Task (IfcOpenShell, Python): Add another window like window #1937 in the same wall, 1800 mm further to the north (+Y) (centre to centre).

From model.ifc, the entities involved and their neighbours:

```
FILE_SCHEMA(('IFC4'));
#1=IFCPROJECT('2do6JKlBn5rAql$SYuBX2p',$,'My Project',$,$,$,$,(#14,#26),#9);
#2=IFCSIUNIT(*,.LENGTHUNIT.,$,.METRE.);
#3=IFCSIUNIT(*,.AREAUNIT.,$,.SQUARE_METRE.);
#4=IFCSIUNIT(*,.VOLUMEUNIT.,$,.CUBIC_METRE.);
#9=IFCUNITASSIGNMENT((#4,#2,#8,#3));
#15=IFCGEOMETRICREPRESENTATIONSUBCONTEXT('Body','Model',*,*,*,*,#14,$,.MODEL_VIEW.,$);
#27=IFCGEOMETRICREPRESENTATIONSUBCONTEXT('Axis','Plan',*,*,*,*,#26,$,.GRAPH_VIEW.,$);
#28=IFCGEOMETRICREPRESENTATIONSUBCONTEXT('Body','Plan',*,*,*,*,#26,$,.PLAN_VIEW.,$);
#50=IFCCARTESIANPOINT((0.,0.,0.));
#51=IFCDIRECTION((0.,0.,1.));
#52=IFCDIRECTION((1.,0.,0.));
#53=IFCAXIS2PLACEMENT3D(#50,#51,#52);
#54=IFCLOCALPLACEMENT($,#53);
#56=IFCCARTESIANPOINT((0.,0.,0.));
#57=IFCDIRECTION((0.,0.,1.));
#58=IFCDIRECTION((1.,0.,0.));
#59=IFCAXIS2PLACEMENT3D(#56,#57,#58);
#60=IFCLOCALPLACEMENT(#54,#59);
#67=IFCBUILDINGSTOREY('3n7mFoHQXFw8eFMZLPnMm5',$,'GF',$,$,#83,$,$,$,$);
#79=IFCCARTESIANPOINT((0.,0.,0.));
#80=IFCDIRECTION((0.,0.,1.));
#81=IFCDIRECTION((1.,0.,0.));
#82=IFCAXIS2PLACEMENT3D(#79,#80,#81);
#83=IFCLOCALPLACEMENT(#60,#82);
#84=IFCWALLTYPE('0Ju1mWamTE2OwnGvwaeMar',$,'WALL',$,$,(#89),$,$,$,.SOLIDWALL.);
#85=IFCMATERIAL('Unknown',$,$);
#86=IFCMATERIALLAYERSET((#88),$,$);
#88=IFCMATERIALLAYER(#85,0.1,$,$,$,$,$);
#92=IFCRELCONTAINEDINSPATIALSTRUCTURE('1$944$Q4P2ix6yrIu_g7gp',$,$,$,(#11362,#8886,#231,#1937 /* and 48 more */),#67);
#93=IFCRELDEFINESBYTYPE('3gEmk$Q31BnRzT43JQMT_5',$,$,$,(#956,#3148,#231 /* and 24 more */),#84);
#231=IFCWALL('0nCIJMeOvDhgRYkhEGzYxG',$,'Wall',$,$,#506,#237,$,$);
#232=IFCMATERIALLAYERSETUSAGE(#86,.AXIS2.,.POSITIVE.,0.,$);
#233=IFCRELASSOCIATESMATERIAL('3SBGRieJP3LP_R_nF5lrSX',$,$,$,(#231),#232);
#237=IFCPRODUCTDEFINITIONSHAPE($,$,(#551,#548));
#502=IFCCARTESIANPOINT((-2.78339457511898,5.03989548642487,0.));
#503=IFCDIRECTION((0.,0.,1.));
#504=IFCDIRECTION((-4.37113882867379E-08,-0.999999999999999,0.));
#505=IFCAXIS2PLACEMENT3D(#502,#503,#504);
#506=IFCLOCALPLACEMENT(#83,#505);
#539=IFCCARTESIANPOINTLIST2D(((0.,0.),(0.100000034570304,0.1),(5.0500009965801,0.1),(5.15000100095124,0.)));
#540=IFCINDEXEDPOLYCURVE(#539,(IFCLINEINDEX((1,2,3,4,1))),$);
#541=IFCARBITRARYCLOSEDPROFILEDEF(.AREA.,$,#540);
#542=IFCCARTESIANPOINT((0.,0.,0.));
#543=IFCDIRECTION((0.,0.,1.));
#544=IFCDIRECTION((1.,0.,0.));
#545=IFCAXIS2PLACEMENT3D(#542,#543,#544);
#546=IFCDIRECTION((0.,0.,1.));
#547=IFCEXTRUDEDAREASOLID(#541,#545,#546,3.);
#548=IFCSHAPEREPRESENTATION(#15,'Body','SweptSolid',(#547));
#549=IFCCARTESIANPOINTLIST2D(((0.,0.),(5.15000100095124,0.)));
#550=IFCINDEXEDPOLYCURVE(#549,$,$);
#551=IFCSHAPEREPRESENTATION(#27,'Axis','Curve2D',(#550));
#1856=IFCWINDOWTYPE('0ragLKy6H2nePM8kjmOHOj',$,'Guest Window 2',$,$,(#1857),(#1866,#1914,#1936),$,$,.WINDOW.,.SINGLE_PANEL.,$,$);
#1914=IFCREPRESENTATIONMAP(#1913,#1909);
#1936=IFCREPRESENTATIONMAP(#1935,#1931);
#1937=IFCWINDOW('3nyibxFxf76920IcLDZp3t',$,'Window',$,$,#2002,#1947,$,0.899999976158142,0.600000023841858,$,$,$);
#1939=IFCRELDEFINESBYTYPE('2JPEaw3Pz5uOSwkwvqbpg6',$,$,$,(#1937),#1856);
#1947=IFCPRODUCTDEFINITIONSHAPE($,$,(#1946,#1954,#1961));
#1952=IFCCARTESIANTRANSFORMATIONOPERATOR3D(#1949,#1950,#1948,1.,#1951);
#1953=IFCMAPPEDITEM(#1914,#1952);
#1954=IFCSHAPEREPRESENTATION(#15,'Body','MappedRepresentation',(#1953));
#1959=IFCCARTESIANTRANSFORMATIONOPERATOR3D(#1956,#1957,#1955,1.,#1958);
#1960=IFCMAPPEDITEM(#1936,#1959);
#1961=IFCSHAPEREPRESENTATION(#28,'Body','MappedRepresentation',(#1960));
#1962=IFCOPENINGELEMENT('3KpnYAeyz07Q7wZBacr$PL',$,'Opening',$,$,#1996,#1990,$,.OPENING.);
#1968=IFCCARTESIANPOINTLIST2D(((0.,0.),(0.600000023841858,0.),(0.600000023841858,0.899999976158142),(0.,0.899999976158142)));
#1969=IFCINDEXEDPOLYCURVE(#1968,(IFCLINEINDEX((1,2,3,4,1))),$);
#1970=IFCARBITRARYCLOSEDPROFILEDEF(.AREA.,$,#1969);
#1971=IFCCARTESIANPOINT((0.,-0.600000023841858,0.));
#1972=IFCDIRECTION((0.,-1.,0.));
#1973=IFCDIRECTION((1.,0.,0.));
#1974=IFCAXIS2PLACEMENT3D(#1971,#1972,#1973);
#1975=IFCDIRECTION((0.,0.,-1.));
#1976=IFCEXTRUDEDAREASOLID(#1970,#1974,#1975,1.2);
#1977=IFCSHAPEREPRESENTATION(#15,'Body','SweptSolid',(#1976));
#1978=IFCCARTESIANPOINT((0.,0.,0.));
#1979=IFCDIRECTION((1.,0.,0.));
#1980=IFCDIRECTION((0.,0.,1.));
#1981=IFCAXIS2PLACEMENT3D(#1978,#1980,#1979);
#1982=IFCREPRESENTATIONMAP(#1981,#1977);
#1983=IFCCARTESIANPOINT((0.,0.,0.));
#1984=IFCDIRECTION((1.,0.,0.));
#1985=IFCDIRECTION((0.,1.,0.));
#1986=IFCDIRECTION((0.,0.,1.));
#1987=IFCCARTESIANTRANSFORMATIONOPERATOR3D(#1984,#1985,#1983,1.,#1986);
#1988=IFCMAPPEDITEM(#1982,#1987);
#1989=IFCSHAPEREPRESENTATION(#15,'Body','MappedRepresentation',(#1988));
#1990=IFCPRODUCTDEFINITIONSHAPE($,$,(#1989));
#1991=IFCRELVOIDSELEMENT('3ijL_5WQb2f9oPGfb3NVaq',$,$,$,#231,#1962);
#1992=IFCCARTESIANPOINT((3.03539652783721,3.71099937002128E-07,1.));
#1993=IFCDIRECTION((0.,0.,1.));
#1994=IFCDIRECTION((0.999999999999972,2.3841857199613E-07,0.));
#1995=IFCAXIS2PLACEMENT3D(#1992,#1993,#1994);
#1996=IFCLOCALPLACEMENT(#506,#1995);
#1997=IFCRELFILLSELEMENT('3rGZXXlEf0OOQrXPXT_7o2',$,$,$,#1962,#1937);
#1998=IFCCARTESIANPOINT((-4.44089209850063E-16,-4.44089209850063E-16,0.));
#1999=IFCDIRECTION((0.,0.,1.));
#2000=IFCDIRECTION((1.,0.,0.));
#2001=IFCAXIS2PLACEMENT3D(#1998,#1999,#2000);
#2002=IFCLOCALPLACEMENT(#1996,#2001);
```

```python
import ifcopenshell
import ifcopenshell.api.feature
import ifcopenshell.api.geometry
import ifcopenshell.api.root
import ifcopenshell.geom
import ifcopenshell.util.element
import ifcopenshell.util.placement
import ifcopenshell.util.shape

model = ifcopenshell.open("model.ifc")
settings = ifcopenshell.geom.settings()


def volume(element):
    """Net volume in cubic metres, openings subtracted."""
    shape = ifcopenshell.geom.create_shape(settings, element)
    return ifcopenshell.util.shape.get_volume(shape.geometry)


window = model.by_id(1937)
opening = window.FillsVoids[0].RelatingOpeningElement
wall = opening.VoidsElements[0].RelatingBuildingElement
before = volume(wall)
shift = ifcopenshell.util.placement.get_local_placement(wall.ObjectPlacement)[:3, 0] * -1.8

# copy_class copies the void relationship, type, container and properties, but no geometry.
new_opening = ifcopenshell.api.root.copy_class(model, product=opening)
new_opening.Representation = ifcopenshell.util.element.copy_deep(
    model, opening.Representation, exclude=["IfcGeometricRepresentationContext", "IfcRepresentationMap"]
)
new_window = ifcopenshell.api.root.copy_class(model, product=window)
new_window.Representation = ifcopenshell.util.element.copy_deep(
    model, window.Representation, exclude=["IfcGeometricRepresentationContext", "IfcRepresentationMap"]
)
ifcopenshell.api.feature.add_filling(model, opening=new_opening, element=new_window)

for old, new in ((opening, new_opening), (window, new_window)):
    matrix = ifcopenshell.util.placement.get_local_placement(old.ObjectPlacement)
    matrix[:3, 3] += shift
    ifcopenshell.api.geometry.edit_object_placement(model, product=new, matrix=matrix, is_si=False)

after = volume(wall)

print(f"wall volume {before:.3f} -> {after:.3f} m3")

model.write("model_edited.ifc")
```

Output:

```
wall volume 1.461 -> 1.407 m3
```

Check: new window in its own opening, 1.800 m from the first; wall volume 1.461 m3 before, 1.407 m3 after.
